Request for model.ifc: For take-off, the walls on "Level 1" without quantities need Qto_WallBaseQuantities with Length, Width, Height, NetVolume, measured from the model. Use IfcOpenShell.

First a look at what the model holds.

```python
import ifcopenshell
import ifcopenshell.util.element
import ifcopenshell.util.unit

model = ifcopenshell.open("model.ifc")
print(model.schema)
for unit_type in ("LENGTHUNIT", "AREAUNIT", "VOLUMEUNIT"):
    print(unit_type, ifcopenshell.util.unit.calculate_unit_scale(model, unit_type))
storey = next(s for s in model.by_type("IfcBuildingStorey") if s.Name == "Level 1")
walls = [e for e in ifcopenshell.util.element.get_decomposition(storey) if e.is_a("IfcWall")]
for e in sorted(walls, key=lambda e: e.id()):
    print(e.id(), e.is_a(), e.Name, list(ifcopenshell.util.element.get_psets(e, qtos_only=True)), sep=" | ")
```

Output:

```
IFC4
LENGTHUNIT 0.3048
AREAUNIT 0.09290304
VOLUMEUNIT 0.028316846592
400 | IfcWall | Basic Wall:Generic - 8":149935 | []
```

```python
import ifcopenshell
import ifcopenshell.api.pset
import ifcopenshell.geom
import ifcopenshell.util.element
import ifcopenshell.util.shape
import ifcopenshell.util.unit

model = ifcopenshell.open("model.ifc")
unit_scale = ifcopenshell.util.unit.calculate_unit_scale(model)
volume_scale = ifcopenshell.util.unit.calculate_unit_scale(model, "VOLUMEUNIT")
settings = ifcopenshell.geom.settings()

storey = next(s for s in model.by_type("IfcBuildingStorey") if s.Name == "Level 1")
walls = [e for e in ifcopenshell.util.element.get_decomposition(storey) if e.is_a("IfcWall")]

for e in sorted(walls, key=lambda e: e.id()):
    if ifcopenshell.util.element.get_psets(e, qtos_only=True, should_inherit=False):
        continue
    # Geometry comes back in metres, in the element's own axes.
    shape = ifcopenshell.geom.create_shape(settings, e)
    values = {
        "Length": ifcopenshell.util.shape.get_x(shape.geometry) / unit_scale,
        "Width": ifcopenshell.util.shape.get_y(shape.geometry) / unit_scale,
        "Height": ifcopenshell.util.shape.get_z(shape.geometry) / unit_scale,
        "NetVolume": ifcopenshell.util.shape.get_volume(shape.geometry) / volume_scale,
    }
    qto = ifcopenshell.api.pset.add_qto(model, product=e, name="Qto_WallBaseQuantities")
    ifcopenshell.api.pset.edit_qto(model, qto=qto, properties=values)
    print(e.id(), {k: round(v, 3) for k, v in values.items()})

model.write("model_updated.ifc")
```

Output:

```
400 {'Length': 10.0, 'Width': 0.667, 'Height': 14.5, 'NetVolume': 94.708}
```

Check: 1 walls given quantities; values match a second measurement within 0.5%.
